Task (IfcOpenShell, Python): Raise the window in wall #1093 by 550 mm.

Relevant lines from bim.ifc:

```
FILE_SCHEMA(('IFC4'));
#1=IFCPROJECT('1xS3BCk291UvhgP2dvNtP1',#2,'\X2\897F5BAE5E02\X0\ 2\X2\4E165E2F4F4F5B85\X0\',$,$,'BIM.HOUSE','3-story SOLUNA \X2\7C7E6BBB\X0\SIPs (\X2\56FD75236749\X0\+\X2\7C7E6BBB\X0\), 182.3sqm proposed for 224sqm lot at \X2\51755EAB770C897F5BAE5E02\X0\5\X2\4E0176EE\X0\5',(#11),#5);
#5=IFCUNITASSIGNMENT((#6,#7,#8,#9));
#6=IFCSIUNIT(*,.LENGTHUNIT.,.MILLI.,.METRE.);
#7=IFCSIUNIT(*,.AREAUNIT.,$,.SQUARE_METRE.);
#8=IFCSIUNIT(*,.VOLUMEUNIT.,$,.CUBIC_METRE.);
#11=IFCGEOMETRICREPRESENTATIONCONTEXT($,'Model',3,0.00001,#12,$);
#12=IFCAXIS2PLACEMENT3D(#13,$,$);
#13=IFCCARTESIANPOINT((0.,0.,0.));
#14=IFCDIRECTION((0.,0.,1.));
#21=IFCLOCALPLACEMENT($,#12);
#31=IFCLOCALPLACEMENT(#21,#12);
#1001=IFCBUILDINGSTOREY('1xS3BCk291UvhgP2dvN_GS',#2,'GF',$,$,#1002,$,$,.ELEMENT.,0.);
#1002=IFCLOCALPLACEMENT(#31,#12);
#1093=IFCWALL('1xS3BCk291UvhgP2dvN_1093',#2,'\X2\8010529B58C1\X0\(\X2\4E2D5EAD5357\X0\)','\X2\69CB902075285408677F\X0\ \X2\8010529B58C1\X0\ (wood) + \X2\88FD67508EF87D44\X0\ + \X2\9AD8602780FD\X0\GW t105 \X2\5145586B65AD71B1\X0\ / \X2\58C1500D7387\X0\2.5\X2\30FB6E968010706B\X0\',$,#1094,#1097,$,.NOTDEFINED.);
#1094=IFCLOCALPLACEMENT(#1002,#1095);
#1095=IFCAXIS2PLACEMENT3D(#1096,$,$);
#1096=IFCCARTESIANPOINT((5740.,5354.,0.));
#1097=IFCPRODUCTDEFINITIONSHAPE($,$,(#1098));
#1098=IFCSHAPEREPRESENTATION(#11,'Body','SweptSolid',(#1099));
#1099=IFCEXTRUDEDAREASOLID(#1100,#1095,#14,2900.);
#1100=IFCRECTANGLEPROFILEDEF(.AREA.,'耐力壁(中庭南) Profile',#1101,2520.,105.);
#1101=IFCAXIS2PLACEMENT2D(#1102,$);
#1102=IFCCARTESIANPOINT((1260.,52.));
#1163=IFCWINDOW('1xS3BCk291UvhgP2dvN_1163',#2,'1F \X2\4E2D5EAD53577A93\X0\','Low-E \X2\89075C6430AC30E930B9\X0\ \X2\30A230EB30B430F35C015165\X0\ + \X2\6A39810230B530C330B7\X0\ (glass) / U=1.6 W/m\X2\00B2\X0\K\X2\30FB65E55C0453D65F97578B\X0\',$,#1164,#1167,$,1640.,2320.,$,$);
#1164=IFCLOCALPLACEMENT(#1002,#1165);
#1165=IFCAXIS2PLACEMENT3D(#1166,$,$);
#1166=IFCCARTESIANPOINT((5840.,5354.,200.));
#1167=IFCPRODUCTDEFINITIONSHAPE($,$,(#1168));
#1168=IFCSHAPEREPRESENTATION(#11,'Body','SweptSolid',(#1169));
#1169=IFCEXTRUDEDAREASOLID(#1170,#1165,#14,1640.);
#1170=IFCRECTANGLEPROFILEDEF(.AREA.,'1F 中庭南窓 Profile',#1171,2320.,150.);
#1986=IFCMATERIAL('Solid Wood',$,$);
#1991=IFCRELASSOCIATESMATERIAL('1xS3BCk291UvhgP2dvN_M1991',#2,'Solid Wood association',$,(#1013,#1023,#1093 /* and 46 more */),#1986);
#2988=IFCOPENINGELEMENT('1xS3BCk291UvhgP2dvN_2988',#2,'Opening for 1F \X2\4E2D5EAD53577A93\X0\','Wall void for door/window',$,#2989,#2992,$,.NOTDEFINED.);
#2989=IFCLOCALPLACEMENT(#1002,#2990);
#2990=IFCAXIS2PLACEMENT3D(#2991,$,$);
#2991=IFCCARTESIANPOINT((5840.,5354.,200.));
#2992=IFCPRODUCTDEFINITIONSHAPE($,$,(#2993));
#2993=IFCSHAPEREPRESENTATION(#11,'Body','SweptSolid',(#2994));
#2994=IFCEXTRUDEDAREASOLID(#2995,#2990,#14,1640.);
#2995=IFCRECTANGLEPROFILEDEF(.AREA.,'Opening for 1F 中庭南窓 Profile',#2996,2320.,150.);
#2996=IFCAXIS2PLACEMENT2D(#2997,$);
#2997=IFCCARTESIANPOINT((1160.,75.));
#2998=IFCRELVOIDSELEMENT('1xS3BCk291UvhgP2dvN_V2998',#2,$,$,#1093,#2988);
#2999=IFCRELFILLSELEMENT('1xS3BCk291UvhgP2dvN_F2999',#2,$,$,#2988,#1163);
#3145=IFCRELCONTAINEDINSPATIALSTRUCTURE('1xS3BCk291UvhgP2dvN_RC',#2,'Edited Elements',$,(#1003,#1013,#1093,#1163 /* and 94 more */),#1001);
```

```python
import numpy as np
import ifcopenshell
import ifcopenshell.api.geometry
import ifcopenshell.util.placement
import ifcopenshell.util.unit

model = ifcopenshell.open("bim.ifc")
unit_scale = ifcopenshell.util.unit.calculate_unit_scale(model)

window = model.by_id(1163)
opening = window.FillsVoids[0].RelatingOpeningElement
dz = 550.0

shift = np.array([0.0, 0.0, dz])
# The window is not placed relative to its opening, so move both.
for product in (opening, window):
    matrix = ifcopenshell.util.placement.get_local_placement(product.ObjectPlacement)
    matrix[:3, 3] += shift
    ifcopenshell.api.geometry.edit_object_placement(model, product=product, matrix=matrix, is_si=False)

print(f"moved by {dz * unit_scale:+.3f} m")

model.write("bim_v2.ifc")
```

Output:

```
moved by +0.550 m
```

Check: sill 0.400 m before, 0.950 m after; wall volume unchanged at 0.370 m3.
